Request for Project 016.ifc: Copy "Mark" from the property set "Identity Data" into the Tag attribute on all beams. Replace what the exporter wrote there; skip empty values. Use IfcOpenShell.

First a look at what the model holds.

```python
import ifcopenshell
import ifcopenshell.util.element

model = ifcopenshell.open("Project 016.ifc")
print(model.schema)
beams = model.by_type("IfcBeam")
print(len(beams), "beams")
for e in beams[:8]:
    source = ifcopenshell.util.element.get_pset(e, "Identity Data", "Mark")
    target = e.Tag
    print(e.id(), repr(source), repr(target), sep=" | ")
```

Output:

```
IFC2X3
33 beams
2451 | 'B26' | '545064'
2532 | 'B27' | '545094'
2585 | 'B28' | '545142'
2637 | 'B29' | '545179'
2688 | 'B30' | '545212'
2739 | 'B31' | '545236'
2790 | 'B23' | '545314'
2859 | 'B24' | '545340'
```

```python
import ifcopenshell
import ifcopenshell.util.element

model = ifcopenshell.open("Project 016.ifc")

count = 0
for e in model.by_type("IfcBeam"):
    value = ifcopenshell.util.element.get_pset(e, "Identity Data", "Mark")
    current = e.Tag
    if not value or not value.strip() or current == value:
        continue
    e.Tag = value
    count += 1

print(count, "beams updated")

model.write("Project 016_rev.ifc")
```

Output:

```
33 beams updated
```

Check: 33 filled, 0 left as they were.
